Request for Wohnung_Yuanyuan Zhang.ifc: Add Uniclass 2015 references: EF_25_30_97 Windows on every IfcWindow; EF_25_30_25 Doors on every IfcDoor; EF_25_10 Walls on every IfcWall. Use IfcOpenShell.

First a look at what the model holds.

```python
import ifcopenshell

model = ifcopenshell.open("Wohnung_Yuanyuan Zhang.ifc")
print(model.schema)
print("classifications:", [c.Name for c in model.by_type("IfcClassification")])
for ifc_class in ("IfcDoor", "IfcRoof", "IfcStair", "IfcWall", "IfcWindow"):
    print(ifc_class, len(model.by_type(ifc_class)))
```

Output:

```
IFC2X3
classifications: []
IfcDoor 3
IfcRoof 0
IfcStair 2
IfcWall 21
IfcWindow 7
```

```python
import ifcopenshell
import ifcopenshell.api.classification

model = ifcopenshell.open("Wohnung_Yuanyuan Zhang.ifc")

# IFC2X3 requires Source and Edition and has no link from the project to the system.
system = model.create_entity("IfcClassification", Source="NBS", Edition="2015", Name="Uniclass 2015")

codes = {
    "IfcWindow": ("EF_25_30_97", "Windows"),
    "IfcDoor": ("EF_25_30_25", "Doors"),
    "IfcWall": ("EF_25_10", "Walls"),
}
for ifc_class, (code, name) in codes.items():
    products = model.by_type(ifc_class)
    ifcopenshell.api.classification.add_reference(
        model, products=products, classification=system, identification=code, name=name
    )
    print(code, len(products))

model.write("Wohnung_Yuanyuan Zhang-out.ifc")
```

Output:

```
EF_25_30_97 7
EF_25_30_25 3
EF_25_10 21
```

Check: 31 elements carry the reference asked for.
